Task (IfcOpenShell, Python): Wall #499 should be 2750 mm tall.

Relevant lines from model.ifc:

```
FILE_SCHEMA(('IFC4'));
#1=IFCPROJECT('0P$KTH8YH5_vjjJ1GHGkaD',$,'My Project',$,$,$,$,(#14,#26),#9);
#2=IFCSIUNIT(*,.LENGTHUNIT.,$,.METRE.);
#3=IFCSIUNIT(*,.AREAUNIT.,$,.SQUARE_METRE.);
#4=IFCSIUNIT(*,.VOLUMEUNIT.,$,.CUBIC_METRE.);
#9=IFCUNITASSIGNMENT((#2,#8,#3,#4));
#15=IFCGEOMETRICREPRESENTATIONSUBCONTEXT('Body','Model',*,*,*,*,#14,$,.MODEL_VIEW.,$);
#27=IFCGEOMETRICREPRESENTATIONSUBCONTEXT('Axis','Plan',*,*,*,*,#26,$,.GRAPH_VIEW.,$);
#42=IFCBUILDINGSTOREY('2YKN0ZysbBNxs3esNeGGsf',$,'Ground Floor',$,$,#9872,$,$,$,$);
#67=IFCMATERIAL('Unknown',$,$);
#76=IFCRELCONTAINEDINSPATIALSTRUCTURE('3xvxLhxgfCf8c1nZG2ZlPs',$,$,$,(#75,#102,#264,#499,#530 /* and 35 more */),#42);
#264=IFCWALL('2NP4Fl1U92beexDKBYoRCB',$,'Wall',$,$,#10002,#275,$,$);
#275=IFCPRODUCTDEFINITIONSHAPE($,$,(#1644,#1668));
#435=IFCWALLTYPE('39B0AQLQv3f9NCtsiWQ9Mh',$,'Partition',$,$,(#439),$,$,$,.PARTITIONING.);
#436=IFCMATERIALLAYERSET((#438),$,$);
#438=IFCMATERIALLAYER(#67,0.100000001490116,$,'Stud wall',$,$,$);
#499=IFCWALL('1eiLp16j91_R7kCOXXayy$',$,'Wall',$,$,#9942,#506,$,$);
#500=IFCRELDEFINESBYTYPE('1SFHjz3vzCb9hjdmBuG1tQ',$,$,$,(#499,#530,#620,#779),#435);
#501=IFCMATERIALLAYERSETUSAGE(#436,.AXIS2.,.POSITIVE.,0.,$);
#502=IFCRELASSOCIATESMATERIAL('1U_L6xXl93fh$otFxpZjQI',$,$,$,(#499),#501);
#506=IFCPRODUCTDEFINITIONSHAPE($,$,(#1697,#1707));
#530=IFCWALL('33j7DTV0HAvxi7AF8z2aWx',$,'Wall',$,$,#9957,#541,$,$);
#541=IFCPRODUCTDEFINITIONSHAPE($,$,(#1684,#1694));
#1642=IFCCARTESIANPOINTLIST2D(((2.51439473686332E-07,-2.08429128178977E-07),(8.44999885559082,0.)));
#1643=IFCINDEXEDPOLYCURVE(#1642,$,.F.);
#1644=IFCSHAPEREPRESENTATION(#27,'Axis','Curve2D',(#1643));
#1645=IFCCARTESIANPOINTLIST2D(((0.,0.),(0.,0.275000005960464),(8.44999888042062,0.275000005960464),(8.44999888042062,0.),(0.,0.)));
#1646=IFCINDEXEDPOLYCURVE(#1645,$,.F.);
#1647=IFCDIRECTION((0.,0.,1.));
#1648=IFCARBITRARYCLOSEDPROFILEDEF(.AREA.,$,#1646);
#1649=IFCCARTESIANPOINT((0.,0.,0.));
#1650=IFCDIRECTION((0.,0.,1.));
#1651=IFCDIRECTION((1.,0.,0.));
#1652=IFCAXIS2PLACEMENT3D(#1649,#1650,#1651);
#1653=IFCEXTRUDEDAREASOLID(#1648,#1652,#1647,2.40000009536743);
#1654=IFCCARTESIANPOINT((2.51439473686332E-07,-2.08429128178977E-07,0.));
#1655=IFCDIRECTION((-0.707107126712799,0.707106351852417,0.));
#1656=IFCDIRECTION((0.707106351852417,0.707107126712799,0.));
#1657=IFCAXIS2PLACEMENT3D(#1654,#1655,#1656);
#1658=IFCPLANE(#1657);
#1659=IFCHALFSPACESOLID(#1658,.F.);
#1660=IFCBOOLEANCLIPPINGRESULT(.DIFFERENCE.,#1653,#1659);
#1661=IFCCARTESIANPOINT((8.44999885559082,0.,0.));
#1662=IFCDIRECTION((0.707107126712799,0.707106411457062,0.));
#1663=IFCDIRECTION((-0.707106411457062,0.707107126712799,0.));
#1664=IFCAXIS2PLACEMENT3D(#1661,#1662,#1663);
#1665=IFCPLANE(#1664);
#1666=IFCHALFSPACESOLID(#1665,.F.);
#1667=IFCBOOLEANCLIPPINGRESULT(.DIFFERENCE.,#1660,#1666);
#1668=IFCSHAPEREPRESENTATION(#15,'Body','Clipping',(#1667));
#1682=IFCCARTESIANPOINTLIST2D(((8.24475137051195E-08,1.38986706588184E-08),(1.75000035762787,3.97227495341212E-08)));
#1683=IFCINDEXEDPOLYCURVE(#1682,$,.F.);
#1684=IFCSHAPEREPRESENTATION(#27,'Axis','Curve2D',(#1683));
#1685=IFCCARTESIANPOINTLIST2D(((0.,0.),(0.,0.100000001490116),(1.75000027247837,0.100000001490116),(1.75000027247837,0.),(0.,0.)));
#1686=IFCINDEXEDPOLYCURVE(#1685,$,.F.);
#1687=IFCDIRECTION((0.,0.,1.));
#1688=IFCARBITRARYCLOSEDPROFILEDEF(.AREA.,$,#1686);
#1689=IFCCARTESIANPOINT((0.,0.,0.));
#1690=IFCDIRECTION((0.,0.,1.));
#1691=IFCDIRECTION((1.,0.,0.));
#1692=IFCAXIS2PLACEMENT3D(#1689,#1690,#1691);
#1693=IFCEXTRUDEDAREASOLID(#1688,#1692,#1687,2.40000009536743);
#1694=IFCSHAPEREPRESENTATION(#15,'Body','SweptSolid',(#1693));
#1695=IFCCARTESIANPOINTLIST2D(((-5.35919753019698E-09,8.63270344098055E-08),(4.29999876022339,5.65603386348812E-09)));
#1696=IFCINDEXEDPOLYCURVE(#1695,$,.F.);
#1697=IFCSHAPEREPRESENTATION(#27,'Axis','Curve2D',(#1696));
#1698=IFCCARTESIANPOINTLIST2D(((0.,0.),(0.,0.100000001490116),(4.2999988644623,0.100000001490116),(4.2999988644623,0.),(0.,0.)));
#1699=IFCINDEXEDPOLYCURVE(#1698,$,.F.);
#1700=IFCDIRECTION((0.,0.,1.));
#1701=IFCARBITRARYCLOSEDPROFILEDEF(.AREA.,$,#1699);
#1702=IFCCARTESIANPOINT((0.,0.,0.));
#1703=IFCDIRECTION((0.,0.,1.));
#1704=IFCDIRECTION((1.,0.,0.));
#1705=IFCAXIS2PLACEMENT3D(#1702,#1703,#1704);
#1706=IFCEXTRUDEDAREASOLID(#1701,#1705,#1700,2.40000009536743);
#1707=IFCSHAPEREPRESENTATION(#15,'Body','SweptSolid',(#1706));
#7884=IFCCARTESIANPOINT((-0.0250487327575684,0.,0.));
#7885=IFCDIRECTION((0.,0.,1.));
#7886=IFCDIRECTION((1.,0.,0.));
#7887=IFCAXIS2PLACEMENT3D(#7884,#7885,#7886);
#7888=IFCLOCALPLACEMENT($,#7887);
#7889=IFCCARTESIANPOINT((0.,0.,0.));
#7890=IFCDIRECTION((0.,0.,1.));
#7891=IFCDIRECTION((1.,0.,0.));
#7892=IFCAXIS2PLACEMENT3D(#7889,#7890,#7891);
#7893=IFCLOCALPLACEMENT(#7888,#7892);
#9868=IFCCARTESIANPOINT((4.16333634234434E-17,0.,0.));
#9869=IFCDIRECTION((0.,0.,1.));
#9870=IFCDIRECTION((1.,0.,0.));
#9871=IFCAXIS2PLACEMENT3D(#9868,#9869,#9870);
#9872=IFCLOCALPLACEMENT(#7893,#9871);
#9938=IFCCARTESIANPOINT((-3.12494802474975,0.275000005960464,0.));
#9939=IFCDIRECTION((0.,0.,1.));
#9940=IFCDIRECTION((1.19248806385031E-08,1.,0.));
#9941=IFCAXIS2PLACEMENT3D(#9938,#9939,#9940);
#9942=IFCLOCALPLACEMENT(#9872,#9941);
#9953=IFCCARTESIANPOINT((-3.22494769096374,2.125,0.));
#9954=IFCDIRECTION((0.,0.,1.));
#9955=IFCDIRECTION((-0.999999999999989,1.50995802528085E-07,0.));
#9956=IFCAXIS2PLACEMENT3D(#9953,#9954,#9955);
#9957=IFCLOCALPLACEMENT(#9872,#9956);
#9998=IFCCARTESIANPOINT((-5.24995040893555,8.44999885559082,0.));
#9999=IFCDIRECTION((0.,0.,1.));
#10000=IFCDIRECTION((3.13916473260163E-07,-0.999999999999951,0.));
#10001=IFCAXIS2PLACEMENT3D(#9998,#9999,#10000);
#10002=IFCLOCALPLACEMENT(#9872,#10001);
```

```python
import ifcopenshell
import ifcopenshell.geom
import ifcopenshell.util.representation
import ifcopenshell.util.shape
import ifcopenshell.util.unit

model = ifcopenshell.open("model.ifc")
unit_scale = ifcopenshell.util.unit.calculate_unit_scale(model)
settings = ifcopenshell.geom.settings()


def volume(element):
    """Net volume in cubic metres, openings subtracted."""
    shape = ifcopenshell.geom.create_shape(settings, element)
    return ifcopenshell.util.shape.get_volume(shape.geometry)


wall = model.by_guid("1eiLp16j91_R7kCOXXayy$")
before = volume(wall)

body = ifcopenshell.util.representation.get_representation(wall, "Model", "Body")
solid = body.Items[0]
old_height = solid.Depth
solid.Depth = 2.75 / unit_scale
after = volume(wall)

print(f"height {old_height:g} -> {solid.Depth:g}, volume {before:.3f} -> {after:.3f} m3")

model.write("model_edited.ifc")
```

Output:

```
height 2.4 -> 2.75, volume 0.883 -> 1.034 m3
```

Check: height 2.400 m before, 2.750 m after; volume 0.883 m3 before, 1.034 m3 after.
